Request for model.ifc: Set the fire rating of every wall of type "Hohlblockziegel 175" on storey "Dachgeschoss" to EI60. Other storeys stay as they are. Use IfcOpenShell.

First a look at what the model holds.

```python
import ifcopenshell
import ifcopenshell.util.element

model = ifcopenshell.open("model.ifc")
print(model.schema)
storey = next(s for s in model.by_type("IfcBuildingStorey") if s.Name == "Dachgeschoss")
walls = [e for e in ifcopenshell.util.element.get_decomposition(storey) if e.is_a("IfcWall")]
seen = {}
for e in walls:
    element_type = ifcopenshell.util.element.get_type(e)
    key = (element_type.Name if element_type != e and element_type else None, ifcopenshell.util.element.get_pset(e, "Pset_WallCommon", "FireRating"))
    seen[key] = seen.get(key, 0) + 1
for (name, value), count in sorted(seen.items(), key=str):
    print(count, "x", name, "|", value)
```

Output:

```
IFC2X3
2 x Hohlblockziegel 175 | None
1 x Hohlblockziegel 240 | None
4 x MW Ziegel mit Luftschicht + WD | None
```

```python
import ifcopenshell
import ifcopenshell.api.pset
import ifcopenshell.util.element

model = ifcopenshell.open("model.ifc")

storey = next(s for s in model.by_type("IfcBuildingStorey") if s.Name == "Dachgeschoss")
walls = [e for e in ifcopenshell.util.element.get_decomposition(storey) if e.is_a("IfcWall")]

count = 0
for e in walls:
    element_type = ifcopenshell.util.element.get_type(e)
    if element_type in (None, e) or element_type.Name != "Hohlblockziegel 175":
        continue
    # add_pset returns the element's existing set when there is one.
    pset = ifcopenshell.api.pset.add_pset(model, product=e, name="Pset_WallCommon")
    ifcopenshell.api.pset.edit_pset(model, pset=pset, properties={"FireRating": "EI60"})
    count += 1

print(count, "walls updated")

model.write("model_rev.ifc")
```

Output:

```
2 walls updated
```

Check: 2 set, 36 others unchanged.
